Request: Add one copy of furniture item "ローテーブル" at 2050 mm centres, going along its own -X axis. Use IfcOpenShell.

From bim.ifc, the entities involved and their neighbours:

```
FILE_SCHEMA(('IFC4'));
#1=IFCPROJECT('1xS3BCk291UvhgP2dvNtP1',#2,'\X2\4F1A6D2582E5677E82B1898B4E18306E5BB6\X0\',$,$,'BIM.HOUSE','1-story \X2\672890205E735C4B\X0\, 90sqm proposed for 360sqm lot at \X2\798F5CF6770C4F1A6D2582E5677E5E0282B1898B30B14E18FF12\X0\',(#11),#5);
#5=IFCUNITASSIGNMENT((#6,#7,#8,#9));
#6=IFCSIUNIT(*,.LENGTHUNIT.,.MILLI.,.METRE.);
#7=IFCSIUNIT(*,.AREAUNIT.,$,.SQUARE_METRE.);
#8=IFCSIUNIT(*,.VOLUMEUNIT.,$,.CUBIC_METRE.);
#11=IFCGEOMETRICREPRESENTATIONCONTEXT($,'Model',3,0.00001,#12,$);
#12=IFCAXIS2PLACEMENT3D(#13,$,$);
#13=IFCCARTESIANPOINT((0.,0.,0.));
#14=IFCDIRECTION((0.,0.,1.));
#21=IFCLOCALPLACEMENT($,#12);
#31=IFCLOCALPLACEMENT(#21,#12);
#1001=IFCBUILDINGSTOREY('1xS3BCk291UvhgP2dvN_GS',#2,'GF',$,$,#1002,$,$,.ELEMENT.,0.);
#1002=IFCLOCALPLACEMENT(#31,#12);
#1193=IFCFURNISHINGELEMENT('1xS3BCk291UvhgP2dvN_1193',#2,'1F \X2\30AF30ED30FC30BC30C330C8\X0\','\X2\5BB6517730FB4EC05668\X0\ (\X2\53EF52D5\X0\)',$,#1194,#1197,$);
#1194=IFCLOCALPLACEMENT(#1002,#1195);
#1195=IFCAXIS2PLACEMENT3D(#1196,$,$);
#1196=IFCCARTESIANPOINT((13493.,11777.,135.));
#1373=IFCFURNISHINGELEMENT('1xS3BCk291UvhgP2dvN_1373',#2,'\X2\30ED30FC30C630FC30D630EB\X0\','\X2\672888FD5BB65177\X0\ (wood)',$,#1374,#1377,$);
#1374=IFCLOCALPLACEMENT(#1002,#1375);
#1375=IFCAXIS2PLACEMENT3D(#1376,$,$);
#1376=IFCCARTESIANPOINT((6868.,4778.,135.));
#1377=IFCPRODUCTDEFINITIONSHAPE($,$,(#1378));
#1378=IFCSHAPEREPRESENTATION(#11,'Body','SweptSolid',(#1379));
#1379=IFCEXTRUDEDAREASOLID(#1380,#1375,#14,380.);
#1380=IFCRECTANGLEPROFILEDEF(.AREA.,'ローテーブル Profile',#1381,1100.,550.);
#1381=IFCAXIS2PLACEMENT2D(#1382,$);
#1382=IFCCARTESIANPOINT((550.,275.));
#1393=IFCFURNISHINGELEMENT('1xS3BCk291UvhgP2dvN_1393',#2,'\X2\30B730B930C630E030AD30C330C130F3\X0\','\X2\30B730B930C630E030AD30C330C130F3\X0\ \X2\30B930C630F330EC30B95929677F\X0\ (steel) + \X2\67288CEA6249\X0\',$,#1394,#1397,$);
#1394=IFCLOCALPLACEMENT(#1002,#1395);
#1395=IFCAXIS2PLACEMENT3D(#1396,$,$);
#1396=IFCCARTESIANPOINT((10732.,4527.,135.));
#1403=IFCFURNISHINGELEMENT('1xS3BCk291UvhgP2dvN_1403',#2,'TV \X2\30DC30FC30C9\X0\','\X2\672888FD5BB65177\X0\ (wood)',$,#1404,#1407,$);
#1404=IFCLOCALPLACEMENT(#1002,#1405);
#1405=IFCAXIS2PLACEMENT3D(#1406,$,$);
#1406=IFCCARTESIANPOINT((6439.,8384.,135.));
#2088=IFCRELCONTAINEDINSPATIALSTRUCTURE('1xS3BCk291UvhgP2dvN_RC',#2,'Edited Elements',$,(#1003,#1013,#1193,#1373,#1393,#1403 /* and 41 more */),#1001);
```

```python
import ifcopenshell
import ifcopenshell.api.geometry
import ifcopenshell.api.root
import ifcopenshell.util.element
import ifcopenshell.util.placement
import ifcopenshell.util.unit

model = ifcopenshell.open("bim.ifc")
unit_scale = ifcopenshell.util.unit.calculate_unit_scale(model)


def reuse_history(source, copy):
    """copy_class also copies each property set's owner history, people and application; keep the originals."""
    for rel in copy.IsDefinedBy:
        if rel.is_a("IfcRelDefinesByProperties") and (history := rel.RelatingPropertyDefinition.OwnerHistory):
            rel.RelatingPropertyDefinition.OwnerHistory = source.OwnerHistory
            ifcopenshell.util.element.remove_deep2(model, history)


source = model.by_id(1373)
base = ifcopenshell.util.placement.get_local_placement(source.ObjectPlacement)
step = -base[:3, 0] * 2.05 / unit_scale

for i in range(1, 2):
    copy = ifcopenshell.api.root.copy_class(model, product=source)
    copy.Representation = ifcopenshell.util.element.copy_deep(
        model, source.Representation, exclude=["IfcGeometricRepresentationContext", "IfcRepresentationMap"]
    )
    reuse_history(source, copy)
    matrix = base.copy()
    matrix[:3, 3] += i * step
    print("added at", matrix[:3, 3].round(3) + 0.0)
    ifcopenshell.api.geometry.edit_object_placement(model, product=copy, matrix=matrix, is_si=False)

model.write("bim_v2.ifc")
```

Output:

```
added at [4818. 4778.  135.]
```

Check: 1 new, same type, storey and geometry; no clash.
